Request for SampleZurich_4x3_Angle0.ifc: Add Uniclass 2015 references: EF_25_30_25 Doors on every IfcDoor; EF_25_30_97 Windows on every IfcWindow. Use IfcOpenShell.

First a look at what the model holds.

```python
import ifcopenshell

model = ifcopenshell.open("SampleZurich_4x3_Angle0.ifc")
print(model.schema)
print("classifications:", [c.Name for c in model.by_type("IfcClassification")])
for ifc_class in ("IfcDoor", "IfcRoof", "IfcStair", "IfcWall", "IfcWindow"):
    print(ifc_class, len(model.by_type(ifc_class)))
```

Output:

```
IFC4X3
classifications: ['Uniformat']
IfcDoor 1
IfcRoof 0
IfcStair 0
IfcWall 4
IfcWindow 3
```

```python
import ifcopenshell
import ifcopenshell.api.classification

model = ifcopenshell.open("SampleZurich_4x3_Angle0.ifc")

system = ifcopenshell.api.classification.add_classification(model, classification="Uniclass 2015")

codes = {
    "IfcDoor": ("EF_25_30_25", "Doors"),
    "IfcWindow": ("EF_25_30_97", "Windows"),
}
for ifc_class, (code, name) in codes.items():
    products = model.by_type(ifc_class)
    ifcopenshell.api.classification.add_reference(
        model, products=products, classification=system, identification=code, name=name
    )
    print(code, len(products))

model.write("SampleZurich_4x3_Angle0-out.ifc")
```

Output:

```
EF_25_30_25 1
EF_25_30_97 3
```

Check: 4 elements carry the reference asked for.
